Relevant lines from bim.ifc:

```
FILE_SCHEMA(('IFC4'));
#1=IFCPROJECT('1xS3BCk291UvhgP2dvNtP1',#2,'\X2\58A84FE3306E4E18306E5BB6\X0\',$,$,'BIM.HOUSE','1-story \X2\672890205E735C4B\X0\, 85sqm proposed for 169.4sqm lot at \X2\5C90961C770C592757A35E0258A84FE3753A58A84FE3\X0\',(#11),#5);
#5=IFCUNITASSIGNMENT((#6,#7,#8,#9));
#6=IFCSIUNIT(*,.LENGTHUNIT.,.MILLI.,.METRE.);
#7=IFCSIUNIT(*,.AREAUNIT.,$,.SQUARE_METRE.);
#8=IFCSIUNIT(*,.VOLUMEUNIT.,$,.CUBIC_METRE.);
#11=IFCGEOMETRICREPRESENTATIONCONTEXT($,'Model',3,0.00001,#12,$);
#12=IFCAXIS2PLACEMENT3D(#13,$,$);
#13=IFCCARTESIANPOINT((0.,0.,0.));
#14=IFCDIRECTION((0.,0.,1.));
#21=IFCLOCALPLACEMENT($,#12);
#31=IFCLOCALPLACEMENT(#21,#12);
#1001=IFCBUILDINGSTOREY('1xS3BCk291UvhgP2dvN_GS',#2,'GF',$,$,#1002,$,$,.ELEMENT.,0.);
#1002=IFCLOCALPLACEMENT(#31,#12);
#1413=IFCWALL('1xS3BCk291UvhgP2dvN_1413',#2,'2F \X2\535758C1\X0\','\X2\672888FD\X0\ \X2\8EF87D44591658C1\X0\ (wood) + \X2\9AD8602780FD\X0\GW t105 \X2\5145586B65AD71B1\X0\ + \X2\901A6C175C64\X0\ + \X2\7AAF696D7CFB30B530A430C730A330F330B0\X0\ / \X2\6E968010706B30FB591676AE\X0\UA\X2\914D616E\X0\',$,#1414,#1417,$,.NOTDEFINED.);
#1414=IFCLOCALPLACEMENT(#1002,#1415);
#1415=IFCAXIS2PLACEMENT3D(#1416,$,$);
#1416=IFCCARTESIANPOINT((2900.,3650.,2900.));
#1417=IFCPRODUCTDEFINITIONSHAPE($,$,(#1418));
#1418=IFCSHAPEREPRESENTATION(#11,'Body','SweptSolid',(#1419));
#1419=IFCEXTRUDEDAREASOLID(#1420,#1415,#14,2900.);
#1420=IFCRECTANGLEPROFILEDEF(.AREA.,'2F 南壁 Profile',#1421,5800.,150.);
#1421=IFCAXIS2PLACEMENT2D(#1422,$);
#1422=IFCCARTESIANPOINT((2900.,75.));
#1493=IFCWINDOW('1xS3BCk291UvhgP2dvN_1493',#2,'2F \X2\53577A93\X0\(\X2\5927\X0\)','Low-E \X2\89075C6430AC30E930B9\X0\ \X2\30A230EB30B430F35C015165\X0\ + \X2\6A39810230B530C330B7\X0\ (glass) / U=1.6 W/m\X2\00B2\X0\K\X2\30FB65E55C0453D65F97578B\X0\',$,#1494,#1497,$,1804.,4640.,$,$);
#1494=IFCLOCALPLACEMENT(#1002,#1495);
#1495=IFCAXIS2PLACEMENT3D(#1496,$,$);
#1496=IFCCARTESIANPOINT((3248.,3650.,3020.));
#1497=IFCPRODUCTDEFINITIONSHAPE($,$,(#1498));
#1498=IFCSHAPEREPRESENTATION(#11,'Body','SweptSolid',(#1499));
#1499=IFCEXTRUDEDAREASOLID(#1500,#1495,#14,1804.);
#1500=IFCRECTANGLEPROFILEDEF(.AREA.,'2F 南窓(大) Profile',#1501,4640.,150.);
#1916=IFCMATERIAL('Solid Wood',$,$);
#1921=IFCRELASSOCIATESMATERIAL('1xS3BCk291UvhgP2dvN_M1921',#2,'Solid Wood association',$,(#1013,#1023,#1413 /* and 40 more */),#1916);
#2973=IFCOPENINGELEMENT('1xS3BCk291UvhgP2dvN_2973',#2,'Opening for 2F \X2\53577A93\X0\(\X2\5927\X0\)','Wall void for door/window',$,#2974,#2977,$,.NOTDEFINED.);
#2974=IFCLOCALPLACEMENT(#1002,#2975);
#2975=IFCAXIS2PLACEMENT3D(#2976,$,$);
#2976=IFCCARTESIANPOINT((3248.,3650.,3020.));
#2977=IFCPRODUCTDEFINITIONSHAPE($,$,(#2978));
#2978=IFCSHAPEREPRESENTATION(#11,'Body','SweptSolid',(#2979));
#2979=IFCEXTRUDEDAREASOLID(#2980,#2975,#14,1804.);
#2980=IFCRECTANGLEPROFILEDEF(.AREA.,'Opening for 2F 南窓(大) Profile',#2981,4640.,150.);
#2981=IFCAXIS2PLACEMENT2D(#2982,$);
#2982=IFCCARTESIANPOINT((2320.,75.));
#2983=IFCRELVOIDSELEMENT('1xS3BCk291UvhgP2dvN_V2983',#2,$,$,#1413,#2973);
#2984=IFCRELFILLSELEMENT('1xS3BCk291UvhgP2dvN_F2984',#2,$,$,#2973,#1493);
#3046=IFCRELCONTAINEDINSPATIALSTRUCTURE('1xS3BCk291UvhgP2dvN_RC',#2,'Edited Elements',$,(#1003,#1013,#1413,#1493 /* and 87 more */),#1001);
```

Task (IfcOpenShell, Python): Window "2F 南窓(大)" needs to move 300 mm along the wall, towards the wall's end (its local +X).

```python
import ifcopenshell
import ifcopenshell.api.geometry
import ifcopenshell.util.placement
import ifcopenshell.util.unit

model = ifcopenshell.open("bim.ifc")
unit_scale = ifcopenshell.util.unit.calculate_unit_scale(model)

window = model.by_guid("1xS3BCk291UvhgP2dvN_1493")
opening = window.FillsVoids[0].RelatingOpeningElement
wall = opening.VoidsElements[0].RelatingBuildingElement

wall_matrix = ifcopenshell.util.placement.get_local_placement(wall.ObjectPlacement)
shift = wall_matrix[:3, 0] * 0.3 / unit_scale
before = ifcopenshell.util.placement.get_local_placement(window.ObjectPlacement)[:3, 3].copy()

# The window is not placed relative to its opening, so move both.
for product in (opening, window):
    matrix = ifcopenshell.util.placement.get_local_placement(product.ObjectPlacement)
    matrix[:3, 3] += shift
    ifcopenshell.api.geometry.edit_object_placement(model, product=product, matrix=matrix, is_si=False)

after = ifcopenshell.util.placement.get_local_placement(window.ObjectPlacement)[:3, 3]
print("window moved by", (after - before).round(3) + 0.0)

model.write("bim_updated.ifc")
```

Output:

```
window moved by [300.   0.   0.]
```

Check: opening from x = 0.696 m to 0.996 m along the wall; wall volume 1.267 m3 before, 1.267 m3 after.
